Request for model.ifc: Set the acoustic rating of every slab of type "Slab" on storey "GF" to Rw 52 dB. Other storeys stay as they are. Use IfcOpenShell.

First a look at what the model holds.

```python
import ifcopenshell
import ifcopenshell.util.element

model = ifcopenshell.open("model.ifc")
print(model.schema)
storey = next(s for s in model.by_type("IfcBuildingStorey") if s.Name == "GF")
slabs = [e for e in ifcopenshell.util.element.get_decomposition(storey) if e.is_a("IfcSlab")]
seen = {}
for e in slabs:
    element_type = ifcopenshell.util.element.get_type(e)
    key = (element_type.Name if element_type != e and element_type else None, ifcopenshell.util.element.get_pset(e, "Pset_SlabCommon", "AcousticRating"))
    seen[key] = seen.get(key, 0) + 1
for (name, value), count in sorted(seen.items(), key=str):
    print(count, "x", name, "|", value)
```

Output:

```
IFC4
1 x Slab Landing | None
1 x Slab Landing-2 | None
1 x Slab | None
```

```python
import ifcopenshell
import ifcopenshell.api.pset
import ifcopenshell.util.element

model = ifcopenshell.open("model.ifc")

storey = next(s for s in model.by_type("IfcBuildingStorey") if s.Name == "GF")
slabs = [e for e in ifcopenshell.util.element.get_decomposition(storey) if e.is_a("IfcSlab")]

count = 0
for e in slabs:
    element_type = ifcopenshell.util.element.get_type(e)
    if element_type in (None, e) or element_type.Name != "Slab":
        continue
    # add_pset returns the element's existing set when there is one.
    pset = ifcopenshell.api.pset.add_pset(model, product=e, name="Pset_SlabCommon")
    ifcopenshell.api.pset.edit_pset(model, pset=pset, properties={"AcousticRating": "Rw 52 dB"})
    count += 1

print(count, "slabs updated")

model.write("model_v2.ifc")
```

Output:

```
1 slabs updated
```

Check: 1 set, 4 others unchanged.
